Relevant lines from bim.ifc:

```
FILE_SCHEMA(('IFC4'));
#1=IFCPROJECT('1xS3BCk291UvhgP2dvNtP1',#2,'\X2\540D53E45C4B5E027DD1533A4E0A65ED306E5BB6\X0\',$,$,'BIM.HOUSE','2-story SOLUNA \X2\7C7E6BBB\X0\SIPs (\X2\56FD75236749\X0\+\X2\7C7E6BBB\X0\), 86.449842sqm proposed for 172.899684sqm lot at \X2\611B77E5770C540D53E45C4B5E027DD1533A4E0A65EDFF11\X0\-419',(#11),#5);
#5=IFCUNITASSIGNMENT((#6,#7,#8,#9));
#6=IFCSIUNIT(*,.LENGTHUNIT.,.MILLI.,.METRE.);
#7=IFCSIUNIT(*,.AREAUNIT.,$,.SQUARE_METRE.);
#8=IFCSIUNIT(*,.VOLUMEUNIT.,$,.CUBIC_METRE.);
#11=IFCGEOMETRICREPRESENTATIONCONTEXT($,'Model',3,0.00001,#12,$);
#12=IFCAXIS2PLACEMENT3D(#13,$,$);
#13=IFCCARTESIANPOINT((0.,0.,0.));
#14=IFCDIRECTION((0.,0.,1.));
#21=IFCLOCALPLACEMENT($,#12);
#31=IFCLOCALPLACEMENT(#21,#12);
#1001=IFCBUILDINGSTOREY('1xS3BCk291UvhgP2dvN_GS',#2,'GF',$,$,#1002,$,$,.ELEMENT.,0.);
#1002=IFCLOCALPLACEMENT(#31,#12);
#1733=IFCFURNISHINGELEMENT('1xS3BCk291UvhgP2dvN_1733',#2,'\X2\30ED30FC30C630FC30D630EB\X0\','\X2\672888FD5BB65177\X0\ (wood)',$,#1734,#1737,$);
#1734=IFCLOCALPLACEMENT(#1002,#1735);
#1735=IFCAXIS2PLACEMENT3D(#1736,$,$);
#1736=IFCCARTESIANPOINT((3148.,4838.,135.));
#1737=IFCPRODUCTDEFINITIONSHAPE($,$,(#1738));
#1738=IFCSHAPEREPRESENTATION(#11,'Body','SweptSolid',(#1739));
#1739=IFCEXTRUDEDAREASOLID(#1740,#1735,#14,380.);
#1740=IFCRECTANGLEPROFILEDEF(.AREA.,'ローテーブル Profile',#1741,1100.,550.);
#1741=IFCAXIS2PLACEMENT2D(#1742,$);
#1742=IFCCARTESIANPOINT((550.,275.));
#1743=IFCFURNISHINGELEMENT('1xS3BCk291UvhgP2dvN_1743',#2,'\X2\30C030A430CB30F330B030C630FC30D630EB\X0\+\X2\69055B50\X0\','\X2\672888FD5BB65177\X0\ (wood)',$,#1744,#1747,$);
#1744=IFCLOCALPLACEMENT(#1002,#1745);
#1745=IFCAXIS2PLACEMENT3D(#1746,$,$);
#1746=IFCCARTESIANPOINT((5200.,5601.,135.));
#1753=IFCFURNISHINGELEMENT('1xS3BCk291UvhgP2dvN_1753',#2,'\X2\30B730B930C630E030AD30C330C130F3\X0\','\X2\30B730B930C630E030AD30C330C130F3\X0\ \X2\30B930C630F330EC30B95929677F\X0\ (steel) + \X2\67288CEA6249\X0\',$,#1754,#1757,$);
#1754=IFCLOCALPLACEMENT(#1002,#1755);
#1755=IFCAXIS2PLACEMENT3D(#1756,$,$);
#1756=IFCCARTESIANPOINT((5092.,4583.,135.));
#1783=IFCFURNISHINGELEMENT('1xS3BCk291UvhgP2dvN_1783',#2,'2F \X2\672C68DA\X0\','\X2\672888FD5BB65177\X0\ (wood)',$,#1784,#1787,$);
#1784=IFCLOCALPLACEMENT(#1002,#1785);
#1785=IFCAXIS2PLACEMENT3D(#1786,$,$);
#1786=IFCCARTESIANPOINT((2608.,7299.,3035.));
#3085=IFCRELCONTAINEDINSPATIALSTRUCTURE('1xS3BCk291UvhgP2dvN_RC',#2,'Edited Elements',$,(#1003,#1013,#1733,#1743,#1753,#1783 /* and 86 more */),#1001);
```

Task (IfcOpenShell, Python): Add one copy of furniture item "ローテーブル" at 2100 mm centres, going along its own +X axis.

```python
import ifcopenshell
import ifcopenshell.api.geometry
import ifcopenshell.api.root
import ifcopenshell.util.element
import ifcopenshell.util.placement
import ifcopenshell.util.unit

model = ifcopenshell.open("bim.ifc")
unit_scale = ifcopenshell.util.unit.calculate_unit_scale(model)


def reuse_history(source, copy):
    """copy_class also copies each property set's owner history, people and application; keep the originals."""
    for rel in copy.IsDefinedBy:
        if rel.is_a("IfcRelDefinesByProperties") and (history := rel.RelatingPropertyDefinition.OwnerHistory):
            rel.RelatingPropertyDefinition.OwnerHistory = source.OwnerHistory
            ifcopenshell.util.element.remove_deep2(model, history)


source = model.by_id(1733)
base = ifcopenshell.util.placement.get_local_placement(source.ObjectPlacement)
step = base[:3, 0] * 2.1 / unit_scale

for i in range(1, 2):
    copy = ifcopenshell.api.root.copy_class(model, product=source)
    copy.Representation = ifcopenshell.util.element.copy_deep(
        model, source.Representation, exclude=["IfcGeometricRepresentationContext", "IfcRepresentationMap"]
    )
    reuse_history(source, copy)
    matrix = base.copy()
    matrix[:3, 3] += i * step
    print("added at", matrix[:3, 3].round(3) + 0.0)
    ifcopenshell.api.geometry.edit_object_placement(model, product=copy, matrix=matrix, is_si=False)

model.write("bim-out.ifc")
```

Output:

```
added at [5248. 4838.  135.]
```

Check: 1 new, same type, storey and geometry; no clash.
